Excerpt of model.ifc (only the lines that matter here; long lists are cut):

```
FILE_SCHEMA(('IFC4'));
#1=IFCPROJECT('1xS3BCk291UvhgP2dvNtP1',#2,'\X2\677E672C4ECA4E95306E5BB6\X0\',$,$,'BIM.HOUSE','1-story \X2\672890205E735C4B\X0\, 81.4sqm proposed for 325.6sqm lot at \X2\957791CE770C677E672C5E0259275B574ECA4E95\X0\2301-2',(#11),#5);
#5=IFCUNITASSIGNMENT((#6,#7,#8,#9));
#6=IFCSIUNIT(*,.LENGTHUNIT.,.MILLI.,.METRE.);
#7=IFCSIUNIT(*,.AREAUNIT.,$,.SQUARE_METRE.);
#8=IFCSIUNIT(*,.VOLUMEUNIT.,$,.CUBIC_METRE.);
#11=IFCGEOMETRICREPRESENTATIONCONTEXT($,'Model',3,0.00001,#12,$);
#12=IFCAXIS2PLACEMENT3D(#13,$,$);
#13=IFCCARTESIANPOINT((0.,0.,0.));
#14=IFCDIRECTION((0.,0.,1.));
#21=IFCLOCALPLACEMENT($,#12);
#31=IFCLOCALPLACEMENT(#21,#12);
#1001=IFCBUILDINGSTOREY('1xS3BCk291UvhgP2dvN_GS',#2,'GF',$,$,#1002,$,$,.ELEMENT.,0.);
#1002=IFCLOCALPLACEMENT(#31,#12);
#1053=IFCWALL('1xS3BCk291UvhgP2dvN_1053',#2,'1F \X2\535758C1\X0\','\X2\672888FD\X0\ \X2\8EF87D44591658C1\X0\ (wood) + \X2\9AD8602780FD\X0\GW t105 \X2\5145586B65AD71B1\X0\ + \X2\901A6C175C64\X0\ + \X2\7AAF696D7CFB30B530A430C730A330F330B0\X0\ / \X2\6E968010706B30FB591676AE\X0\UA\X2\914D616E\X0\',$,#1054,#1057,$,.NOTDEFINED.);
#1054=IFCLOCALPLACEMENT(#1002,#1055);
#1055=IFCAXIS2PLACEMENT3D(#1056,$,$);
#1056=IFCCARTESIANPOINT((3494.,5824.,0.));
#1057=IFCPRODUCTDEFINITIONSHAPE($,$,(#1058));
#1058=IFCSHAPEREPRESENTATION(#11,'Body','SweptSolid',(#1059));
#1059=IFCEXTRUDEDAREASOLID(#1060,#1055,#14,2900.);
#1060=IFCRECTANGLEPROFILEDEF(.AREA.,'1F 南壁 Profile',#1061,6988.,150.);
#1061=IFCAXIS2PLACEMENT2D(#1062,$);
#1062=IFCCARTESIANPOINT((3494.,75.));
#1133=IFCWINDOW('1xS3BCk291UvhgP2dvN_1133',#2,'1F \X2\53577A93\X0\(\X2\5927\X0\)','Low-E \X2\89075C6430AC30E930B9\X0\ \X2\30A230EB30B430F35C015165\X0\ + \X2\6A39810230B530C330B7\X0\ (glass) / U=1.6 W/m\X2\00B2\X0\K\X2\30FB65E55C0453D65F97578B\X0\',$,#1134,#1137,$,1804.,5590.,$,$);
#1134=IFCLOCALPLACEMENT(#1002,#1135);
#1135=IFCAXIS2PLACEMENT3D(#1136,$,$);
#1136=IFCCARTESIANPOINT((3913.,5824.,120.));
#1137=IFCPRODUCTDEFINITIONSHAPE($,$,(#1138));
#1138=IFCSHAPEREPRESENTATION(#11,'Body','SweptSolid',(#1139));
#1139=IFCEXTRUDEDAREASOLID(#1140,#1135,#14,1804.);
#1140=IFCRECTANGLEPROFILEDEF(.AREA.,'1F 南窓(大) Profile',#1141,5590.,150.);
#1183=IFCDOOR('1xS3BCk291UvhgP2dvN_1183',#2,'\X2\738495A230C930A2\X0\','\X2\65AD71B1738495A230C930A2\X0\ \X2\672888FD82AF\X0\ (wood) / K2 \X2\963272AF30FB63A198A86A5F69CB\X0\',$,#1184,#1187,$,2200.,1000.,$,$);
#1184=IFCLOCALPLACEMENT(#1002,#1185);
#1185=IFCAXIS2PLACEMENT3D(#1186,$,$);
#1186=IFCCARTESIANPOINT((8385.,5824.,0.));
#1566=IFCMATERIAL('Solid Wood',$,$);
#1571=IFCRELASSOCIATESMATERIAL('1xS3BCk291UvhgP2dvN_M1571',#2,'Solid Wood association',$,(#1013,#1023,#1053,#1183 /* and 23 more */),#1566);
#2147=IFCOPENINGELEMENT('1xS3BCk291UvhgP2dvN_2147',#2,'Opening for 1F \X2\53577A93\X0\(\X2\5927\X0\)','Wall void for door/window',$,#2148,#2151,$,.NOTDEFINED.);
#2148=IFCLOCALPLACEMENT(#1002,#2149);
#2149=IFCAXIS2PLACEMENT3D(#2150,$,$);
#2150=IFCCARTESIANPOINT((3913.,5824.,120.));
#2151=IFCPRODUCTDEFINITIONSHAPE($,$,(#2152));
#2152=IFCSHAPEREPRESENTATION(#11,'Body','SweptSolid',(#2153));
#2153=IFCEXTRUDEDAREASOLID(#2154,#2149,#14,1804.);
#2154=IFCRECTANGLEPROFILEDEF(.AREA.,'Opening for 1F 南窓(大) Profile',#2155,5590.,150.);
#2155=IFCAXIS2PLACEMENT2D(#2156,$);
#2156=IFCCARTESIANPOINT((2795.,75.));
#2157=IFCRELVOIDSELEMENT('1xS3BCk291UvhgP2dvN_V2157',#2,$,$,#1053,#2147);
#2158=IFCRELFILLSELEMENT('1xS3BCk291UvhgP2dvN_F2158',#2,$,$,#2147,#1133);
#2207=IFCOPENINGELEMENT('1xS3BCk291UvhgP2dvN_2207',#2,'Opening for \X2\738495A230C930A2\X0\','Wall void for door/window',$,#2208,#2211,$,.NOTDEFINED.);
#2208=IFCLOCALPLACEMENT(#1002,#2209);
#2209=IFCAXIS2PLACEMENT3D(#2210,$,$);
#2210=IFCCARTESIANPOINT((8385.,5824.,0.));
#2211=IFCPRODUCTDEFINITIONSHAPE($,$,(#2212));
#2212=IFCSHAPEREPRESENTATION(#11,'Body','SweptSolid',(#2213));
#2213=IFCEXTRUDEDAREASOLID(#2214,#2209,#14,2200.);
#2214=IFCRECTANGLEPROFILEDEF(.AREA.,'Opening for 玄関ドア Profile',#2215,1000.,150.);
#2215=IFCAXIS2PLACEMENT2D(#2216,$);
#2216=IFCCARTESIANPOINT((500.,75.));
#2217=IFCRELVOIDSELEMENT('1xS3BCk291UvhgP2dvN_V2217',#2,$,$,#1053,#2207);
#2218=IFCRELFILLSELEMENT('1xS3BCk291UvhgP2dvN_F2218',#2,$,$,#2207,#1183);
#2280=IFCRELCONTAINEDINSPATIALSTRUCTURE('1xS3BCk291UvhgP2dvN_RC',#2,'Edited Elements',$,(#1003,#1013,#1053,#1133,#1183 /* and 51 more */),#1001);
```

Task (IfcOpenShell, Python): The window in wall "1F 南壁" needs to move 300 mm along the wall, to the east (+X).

```python
import ifcopenshell
import ifcopenshell.api.geometry
import ifcopenshell.util.placement
import ifcopenshell.util.unit

model = ifcopenshell.open("model.ifc")
unit_scale = ifcopenshell.util.unit.calculate_unit_scale(model)

window = model.by_guid("1xS3BCk291UvhgP2dvN_1133")
opening = window.FillsVoids[0].RelatingOpeningElement
wall = opening.VoidsElements[0].RelatingBuildingElement

wall_matrix = ifcopenshell.util.placement.get_local_placement(wall.ObjectPlacement)
shift = wall_matrix[:3, 0] * 0.3 / unit_scale
before = ifcopenshell.util.placement.get_local_placement(window.ObjectPlacement)[:3, 3].copy()

# The window is not placed relative to its opening, so move both.
for product in (opening, window):
    matrix = ifcopenshell.util.placement.get_local_placement(product.ObjectPlacement)
    matrix[:3, 3] += shift
    ifcopenshell.api.geometry.edit_object_placement(model, product=product, matrix=matrix, is_si=False)

after = ifcopenshell.util.placement.get_local_placement(window.ObjectPlacement)[:3, 3]
print("window moved by", (after - before).round(3) + 0.0)

model.write("model_updated.ifc")
```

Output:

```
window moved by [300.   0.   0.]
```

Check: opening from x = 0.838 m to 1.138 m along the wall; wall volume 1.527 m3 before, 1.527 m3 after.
